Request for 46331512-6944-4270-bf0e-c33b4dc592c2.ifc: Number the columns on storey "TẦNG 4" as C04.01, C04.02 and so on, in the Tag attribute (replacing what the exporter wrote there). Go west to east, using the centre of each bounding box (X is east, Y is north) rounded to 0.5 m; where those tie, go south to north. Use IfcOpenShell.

First a look at what the model holds.

```python
import ifcopenshell
import ifcopenshell.util.element
import ifcopenshell.util.placement

model = ifcopenshell.open("46331512-6944-4270-bf0e-c33b4dc592c2.ifc")
print(model.schema)
storey = next(s for s in model.by_type("IfcBuildingStorey") if s.Name == "TẦNG 4")
columns = [e for e in ifcopenshell.util.element.get_decomposition(storey) if e.is_a("IfcColumn")]
for e in sorted(columns, key=lambda e: e.id()):
    origin = ifcopenshell.util.placement.get_local_placement(e.ObjectPlacement)[:3, 3]
    print(e.id(), e.Tag, e.Name, origin.round(2) + 0.0, sep=" | ")
```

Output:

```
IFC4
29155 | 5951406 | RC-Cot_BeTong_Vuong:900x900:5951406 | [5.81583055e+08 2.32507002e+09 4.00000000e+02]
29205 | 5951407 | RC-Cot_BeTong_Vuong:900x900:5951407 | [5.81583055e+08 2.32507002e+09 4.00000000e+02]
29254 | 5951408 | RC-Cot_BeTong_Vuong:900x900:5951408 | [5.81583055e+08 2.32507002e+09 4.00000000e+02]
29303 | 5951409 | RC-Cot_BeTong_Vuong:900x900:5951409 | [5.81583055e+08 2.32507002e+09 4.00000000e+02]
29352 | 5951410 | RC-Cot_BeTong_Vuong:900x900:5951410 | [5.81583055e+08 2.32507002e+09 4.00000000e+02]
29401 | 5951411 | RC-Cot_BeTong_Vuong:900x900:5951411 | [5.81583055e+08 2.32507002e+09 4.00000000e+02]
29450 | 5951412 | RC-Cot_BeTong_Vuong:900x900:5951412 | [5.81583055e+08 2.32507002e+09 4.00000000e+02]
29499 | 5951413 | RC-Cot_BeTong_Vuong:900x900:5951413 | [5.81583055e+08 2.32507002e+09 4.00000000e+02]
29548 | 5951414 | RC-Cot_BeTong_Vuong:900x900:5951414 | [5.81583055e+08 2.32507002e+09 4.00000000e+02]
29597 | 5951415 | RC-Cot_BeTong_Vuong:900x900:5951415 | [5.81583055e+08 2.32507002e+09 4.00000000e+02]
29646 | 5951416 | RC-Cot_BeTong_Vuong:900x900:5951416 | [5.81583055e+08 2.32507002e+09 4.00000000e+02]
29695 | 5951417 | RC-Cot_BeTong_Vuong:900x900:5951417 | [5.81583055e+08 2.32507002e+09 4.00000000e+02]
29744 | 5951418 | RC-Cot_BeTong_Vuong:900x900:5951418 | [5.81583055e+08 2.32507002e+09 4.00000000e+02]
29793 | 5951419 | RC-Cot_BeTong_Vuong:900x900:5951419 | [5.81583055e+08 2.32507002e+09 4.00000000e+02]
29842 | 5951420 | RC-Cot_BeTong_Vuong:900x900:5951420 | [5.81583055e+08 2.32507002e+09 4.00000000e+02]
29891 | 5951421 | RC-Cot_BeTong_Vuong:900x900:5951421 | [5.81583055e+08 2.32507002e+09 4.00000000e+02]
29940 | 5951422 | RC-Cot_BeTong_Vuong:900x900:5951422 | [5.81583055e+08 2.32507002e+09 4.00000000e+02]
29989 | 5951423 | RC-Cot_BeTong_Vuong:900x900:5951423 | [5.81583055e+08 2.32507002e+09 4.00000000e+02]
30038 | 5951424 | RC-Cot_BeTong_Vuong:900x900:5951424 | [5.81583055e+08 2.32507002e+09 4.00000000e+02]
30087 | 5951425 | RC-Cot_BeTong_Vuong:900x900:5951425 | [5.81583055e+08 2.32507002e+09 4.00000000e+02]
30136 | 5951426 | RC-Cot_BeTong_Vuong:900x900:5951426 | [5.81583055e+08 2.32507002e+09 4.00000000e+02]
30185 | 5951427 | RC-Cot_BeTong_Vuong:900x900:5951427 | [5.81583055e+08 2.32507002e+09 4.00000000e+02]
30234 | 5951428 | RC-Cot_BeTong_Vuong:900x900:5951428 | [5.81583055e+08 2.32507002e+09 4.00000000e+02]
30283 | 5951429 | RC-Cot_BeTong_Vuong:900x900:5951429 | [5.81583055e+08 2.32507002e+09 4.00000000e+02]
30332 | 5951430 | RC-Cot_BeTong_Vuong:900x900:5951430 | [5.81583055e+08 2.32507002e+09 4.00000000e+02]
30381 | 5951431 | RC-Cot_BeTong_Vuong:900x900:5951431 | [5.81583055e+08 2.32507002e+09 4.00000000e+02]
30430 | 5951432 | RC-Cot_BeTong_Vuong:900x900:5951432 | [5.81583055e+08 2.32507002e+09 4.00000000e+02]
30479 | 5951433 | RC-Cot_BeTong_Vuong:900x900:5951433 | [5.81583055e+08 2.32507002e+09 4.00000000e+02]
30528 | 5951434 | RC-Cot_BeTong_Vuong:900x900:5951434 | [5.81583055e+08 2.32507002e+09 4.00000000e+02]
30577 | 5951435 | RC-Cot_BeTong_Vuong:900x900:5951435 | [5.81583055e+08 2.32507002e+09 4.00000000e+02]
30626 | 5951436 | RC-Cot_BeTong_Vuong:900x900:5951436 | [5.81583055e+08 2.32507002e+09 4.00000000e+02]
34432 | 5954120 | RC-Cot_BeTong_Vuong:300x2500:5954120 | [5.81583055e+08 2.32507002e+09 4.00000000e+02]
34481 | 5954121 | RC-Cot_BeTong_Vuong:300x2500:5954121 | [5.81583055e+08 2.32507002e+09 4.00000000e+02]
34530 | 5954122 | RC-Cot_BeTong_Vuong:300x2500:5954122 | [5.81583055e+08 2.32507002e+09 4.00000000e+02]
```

```python
import ifcopenshell
import ifcopenshell.geom
import ifcopenshell.util.element
import ifcopenshell.util.shape

model = ifcopenshell.open("46331512-6944-4270-bf0e-c33b4dc592c2.ifc")
settings = ifcopenshell.geom.settings()
settings.set("use-world-coords", True)


def centre(element):
    shape = ifcopenshell.geom.create_shape(settings, element)
    return ifcopenshell.util.shape.get_bbox_centroid(shape.geometry)


storey = next(s for s in model.by_type("IfcBuildingStorey") if s.Name == "TẦNG 4")
columns = [e for e in ifcopenshell.util.element.get_decomposition(storey) if e.is_a("IfcColumn")]

# Insertion points can sit at a corner or the storey origin, so sort by the geometry (in metres).
centres = {e: centre(e) for e in columns}
columns.sort(key=lambda e: (round(centres[e][0] / 0.5), centres[e][1]))

for i, e in enumerate(columns, start=1):
    number = f"C04.{i:02d}"
    e.Tag = number
    print(e.id(), number)

model.write("46331512-6944-4270-bf0e-c33b4dc592c2_updated.ifc")
```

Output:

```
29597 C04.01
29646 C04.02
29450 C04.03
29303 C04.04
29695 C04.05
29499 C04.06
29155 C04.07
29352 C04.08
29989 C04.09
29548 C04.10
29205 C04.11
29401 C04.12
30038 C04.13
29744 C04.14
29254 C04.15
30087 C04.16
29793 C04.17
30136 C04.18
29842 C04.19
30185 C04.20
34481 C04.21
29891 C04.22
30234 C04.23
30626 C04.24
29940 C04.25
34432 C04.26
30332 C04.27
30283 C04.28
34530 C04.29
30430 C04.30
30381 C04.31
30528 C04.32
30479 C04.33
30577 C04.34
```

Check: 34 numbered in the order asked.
